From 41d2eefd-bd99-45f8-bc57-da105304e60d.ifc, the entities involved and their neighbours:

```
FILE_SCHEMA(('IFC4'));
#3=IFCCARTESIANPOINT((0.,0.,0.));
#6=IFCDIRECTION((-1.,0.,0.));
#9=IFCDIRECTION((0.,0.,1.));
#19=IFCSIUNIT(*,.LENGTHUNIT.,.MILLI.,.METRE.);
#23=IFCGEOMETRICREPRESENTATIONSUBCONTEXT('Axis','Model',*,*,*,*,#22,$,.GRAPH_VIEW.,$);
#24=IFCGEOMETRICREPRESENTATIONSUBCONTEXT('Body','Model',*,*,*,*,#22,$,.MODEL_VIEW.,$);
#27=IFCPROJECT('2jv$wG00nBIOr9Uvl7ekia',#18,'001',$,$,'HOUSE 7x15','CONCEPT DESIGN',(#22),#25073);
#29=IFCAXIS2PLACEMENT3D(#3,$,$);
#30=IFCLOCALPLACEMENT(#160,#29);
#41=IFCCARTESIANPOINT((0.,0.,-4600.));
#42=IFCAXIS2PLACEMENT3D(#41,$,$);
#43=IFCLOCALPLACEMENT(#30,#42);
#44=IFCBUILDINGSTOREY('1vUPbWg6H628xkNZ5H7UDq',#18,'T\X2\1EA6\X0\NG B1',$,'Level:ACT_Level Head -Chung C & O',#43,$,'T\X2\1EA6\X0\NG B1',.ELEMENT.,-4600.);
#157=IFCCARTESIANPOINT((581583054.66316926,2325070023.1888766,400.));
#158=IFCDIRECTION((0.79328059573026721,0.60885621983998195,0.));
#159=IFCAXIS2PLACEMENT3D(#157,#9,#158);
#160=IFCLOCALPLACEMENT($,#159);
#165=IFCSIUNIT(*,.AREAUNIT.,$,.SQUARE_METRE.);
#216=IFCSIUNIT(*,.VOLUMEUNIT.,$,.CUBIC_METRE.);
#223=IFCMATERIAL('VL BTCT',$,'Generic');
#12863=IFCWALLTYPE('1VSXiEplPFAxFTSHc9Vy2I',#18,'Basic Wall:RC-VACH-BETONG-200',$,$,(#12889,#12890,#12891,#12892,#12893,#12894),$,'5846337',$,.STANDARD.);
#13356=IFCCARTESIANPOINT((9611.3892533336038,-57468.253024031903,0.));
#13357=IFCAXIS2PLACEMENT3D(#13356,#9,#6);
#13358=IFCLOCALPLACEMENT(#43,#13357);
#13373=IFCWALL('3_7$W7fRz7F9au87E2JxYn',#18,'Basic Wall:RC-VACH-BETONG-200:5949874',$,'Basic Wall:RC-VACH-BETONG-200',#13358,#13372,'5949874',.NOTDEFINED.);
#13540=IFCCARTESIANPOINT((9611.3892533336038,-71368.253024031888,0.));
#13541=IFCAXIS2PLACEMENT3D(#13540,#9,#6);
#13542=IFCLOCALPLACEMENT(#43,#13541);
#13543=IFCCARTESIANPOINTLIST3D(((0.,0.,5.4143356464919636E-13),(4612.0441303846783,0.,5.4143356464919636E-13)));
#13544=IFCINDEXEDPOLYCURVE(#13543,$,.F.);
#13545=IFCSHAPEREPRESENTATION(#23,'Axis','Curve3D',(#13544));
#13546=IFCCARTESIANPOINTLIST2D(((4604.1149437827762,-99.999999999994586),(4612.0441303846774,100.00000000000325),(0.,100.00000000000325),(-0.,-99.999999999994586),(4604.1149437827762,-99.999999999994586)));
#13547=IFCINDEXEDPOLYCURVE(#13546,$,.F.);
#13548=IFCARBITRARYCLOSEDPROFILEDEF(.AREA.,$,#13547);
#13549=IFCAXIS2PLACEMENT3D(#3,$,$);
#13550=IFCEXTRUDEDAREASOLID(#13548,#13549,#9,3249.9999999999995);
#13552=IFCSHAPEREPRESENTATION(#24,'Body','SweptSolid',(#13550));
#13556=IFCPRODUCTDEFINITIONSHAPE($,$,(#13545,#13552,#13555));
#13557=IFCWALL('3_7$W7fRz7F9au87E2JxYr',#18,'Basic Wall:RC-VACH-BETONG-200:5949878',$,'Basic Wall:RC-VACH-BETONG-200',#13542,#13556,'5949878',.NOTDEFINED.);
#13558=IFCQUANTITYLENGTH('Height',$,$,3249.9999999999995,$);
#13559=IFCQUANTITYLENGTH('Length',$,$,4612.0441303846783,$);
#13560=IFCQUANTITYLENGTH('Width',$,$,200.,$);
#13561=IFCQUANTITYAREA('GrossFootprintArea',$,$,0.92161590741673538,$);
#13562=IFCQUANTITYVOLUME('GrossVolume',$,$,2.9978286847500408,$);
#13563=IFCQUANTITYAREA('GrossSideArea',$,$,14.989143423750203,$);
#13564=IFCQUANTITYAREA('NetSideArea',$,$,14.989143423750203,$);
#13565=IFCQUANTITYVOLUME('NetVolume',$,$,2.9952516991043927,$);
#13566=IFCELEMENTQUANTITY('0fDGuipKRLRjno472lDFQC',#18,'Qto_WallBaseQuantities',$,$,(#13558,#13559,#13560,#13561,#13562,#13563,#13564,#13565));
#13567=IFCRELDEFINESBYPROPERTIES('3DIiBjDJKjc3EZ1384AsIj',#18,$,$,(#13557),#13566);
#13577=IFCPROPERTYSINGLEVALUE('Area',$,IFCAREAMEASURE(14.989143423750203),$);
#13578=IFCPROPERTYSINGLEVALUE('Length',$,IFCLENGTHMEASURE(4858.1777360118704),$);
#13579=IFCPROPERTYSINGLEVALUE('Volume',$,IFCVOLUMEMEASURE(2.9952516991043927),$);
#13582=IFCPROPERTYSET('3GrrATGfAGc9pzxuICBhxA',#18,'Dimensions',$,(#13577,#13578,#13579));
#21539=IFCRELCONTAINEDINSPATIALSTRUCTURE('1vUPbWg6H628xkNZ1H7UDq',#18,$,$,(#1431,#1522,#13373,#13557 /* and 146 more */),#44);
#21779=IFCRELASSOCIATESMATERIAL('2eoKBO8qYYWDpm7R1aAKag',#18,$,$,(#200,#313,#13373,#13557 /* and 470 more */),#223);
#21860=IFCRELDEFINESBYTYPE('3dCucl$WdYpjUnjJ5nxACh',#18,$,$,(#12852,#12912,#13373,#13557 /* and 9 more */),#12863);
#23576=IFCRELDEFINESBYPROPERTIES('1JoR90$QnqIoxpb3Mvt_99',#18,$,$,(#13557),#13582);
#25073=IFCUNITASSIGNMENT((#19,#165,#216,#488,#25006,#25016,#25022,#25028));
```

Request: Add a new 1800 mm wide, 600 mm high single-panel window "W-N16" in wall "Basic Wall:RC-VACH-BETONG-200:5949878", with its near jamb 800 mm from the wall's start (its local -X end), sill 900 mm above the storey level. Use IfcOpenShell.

```python
import numpy as np
import ifcopenshell
import ifcopenshell.api.feature
import ifcopenshell.api.geometry
import ifcopenshell.api.pset
import ifcopenshell.api.root
import ifcopenshell.api.spatial
import ifcopenshell.geom
import ifcopenshell.util.element
import ifcopenshell.util.placement
import ifcopenshell.util.representation
import ifcopenshell.util.shape
import ifcopenshell.util.unit

model = ifcopenshell.open("41d2eefd-bd99-45f8-bc57-da105304e60d.ifc")
unit_scale = ifcopenshell.util.unit.calculate_unit_scale(model)
area_scale = ifcopenshell.util.unit.calculate_unit_scale(model, "AREAUNIT")
volume_scale = ifcopenshell.util.unit.calculate_unit_scale(model, "VOLUMEUNIT")
settings = ifcopenshell.geom.settings()


def volume(element):
    """Net volume in cubic metres, openings subtracted."""
    shape = ifcopenshell.geom.create_shape(settings, element)
    return ifcopenshell.util.shape.get_volume(shape.geometry)


wall = model.by_id(13557)
storey = ifcopenshell.util.element.get_container(wall, ifc_class="IfcBuildingStorey")
context = ifcopenshell.util.representation.get_context(model, "Model", "Body", "MODEL_VIEW")
before = volume(wall)

width, height, from_end, sill = 1.8, 0.6, 0.8, 0.9  # metres

# The wall runs along its own X axis, and the end named is its -X end.
wall_shape = ifcopenshell.geom.create_shape(settings, wall)
x, y, z = ifcopenshell.util.shape.get_vertices(wall_shape.geometry).T
start = x.min() + from_end
face, thickness = float(y.min()), float(y.max() - y.min())
wall_matrix = ifcopenshell.util.placement.get_local_placement(wall.ObjectPlacement)
level = ifcopenshell.util.placement.get_local_placement(storey.ObjectPlacement)[2, 3]


def in_wall(x, y):
    """Placement at x, y metres in the wall's axes, at sill height."""
    matrix = wall_matrix.copy()
    matrix[:, 3] = wall_matrix @ np.array([x / unit_scale, y / unit_scale, 0.0, 1.0])
    matrix[2, 3] = level + sill / unit_scale
    return matrix


# Opening: a box that overshoots both wall faces by 50 mm.
opening = ifcopenshell.api.root.create_entity(model, ifc_class="IfcOpeningElement", predefined_type="OPENING")
box = ifcopenshell.api.geometry.add_wall_representation(
    model, context=context, length=width, height=height, thickness=thickness + 0.1
)
ifcopenshell.api.geometry.assign_representation(model, product=opening, representation=box)
ifcopenshell.api.geometry.edit_object_placement(model, product=opening, matrix=in_wall(start, face - 0.05), is_si=False)
ifcopenshell.api.feature.add_feature(model, feature=opening, element=wall)

window = ifcopenshell.api.root.create_entity(model, ifc_class="IfcWindow", name="W-N16", predefined_type="WINDOW")
window.OverallWidth, window.OverallHeight = width / unit_scale, height / unit_scale
window.PartitioningType = "SINGLE_PANEL"
body = ifcopenshell.api.geometry.add_window_representation(
    model,
    context=context,
    overall_width=window.OverallWidth,
    overall_height=window.OverallHeight,
    partition_type="SINGLE_PANEL",
)
ifcopenshell.api.geometry.assign_representation(model, product=window, representation=body)
ifcopenshell.api.spatial.assign_container(model, products=[window], relating_structure=storey)
ifcopenshell.api.feature.add_filling(model, opening=opening, element=window)

# Centre the window in the wall's thickness.
ifcopenshell.api.geometry.edit_object_placement(model, product=window, matrix=in_wall(start, face), is_si=False)
window_shape = ifcopenshell.geom.create_shape(settings, window)
depth = ifcopenshell.util.shape.get_vertices(window_shape.geometry)[:, 1]
offset = face + thickness / 2 - (depth.min() + depth.max()) / 2
ifcopenshell.api.geometry.edit_object_placement(model, product=window, matrix=in_wall(start, offset), is_si=False)

after = volume(wall)

# Update the wall's stored quantities.
qto = model.by_id(ifcopenshell.util.element.get_pset(wall, "Qto_WallBaseQuantities", should_inherit=False)["id"])
ifcopenshell.api.pset.edit_qto(model, qto=qto, properties={
    "NetSideArea": after / thickness / area_scale,
    "NetVolume": after / volume_scale,
})
pset = model.by_id(ifcopenshell.util.element.get_pset(wall, "Dimensions", should_inherit=False)["id"])
ifcopenshell.api.pset.edit_pset(model, pset=pset, properties={
    "Area": model.create_entity("IfcAreaMeasure", after / thickness / area_scale),
    "Volume": model.create_entity("IfcVolumeMeasure", after / volume_scale),
})

print(f"wall volume {before:.3f} -> {after:.3f} m3")

model.write("41d2eefd-bd99-45f8-bc57-da105304e60d_v2.ifc")
```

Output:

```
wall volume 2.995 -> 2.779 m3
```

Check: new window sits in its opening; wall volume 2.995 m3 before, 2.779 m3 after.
